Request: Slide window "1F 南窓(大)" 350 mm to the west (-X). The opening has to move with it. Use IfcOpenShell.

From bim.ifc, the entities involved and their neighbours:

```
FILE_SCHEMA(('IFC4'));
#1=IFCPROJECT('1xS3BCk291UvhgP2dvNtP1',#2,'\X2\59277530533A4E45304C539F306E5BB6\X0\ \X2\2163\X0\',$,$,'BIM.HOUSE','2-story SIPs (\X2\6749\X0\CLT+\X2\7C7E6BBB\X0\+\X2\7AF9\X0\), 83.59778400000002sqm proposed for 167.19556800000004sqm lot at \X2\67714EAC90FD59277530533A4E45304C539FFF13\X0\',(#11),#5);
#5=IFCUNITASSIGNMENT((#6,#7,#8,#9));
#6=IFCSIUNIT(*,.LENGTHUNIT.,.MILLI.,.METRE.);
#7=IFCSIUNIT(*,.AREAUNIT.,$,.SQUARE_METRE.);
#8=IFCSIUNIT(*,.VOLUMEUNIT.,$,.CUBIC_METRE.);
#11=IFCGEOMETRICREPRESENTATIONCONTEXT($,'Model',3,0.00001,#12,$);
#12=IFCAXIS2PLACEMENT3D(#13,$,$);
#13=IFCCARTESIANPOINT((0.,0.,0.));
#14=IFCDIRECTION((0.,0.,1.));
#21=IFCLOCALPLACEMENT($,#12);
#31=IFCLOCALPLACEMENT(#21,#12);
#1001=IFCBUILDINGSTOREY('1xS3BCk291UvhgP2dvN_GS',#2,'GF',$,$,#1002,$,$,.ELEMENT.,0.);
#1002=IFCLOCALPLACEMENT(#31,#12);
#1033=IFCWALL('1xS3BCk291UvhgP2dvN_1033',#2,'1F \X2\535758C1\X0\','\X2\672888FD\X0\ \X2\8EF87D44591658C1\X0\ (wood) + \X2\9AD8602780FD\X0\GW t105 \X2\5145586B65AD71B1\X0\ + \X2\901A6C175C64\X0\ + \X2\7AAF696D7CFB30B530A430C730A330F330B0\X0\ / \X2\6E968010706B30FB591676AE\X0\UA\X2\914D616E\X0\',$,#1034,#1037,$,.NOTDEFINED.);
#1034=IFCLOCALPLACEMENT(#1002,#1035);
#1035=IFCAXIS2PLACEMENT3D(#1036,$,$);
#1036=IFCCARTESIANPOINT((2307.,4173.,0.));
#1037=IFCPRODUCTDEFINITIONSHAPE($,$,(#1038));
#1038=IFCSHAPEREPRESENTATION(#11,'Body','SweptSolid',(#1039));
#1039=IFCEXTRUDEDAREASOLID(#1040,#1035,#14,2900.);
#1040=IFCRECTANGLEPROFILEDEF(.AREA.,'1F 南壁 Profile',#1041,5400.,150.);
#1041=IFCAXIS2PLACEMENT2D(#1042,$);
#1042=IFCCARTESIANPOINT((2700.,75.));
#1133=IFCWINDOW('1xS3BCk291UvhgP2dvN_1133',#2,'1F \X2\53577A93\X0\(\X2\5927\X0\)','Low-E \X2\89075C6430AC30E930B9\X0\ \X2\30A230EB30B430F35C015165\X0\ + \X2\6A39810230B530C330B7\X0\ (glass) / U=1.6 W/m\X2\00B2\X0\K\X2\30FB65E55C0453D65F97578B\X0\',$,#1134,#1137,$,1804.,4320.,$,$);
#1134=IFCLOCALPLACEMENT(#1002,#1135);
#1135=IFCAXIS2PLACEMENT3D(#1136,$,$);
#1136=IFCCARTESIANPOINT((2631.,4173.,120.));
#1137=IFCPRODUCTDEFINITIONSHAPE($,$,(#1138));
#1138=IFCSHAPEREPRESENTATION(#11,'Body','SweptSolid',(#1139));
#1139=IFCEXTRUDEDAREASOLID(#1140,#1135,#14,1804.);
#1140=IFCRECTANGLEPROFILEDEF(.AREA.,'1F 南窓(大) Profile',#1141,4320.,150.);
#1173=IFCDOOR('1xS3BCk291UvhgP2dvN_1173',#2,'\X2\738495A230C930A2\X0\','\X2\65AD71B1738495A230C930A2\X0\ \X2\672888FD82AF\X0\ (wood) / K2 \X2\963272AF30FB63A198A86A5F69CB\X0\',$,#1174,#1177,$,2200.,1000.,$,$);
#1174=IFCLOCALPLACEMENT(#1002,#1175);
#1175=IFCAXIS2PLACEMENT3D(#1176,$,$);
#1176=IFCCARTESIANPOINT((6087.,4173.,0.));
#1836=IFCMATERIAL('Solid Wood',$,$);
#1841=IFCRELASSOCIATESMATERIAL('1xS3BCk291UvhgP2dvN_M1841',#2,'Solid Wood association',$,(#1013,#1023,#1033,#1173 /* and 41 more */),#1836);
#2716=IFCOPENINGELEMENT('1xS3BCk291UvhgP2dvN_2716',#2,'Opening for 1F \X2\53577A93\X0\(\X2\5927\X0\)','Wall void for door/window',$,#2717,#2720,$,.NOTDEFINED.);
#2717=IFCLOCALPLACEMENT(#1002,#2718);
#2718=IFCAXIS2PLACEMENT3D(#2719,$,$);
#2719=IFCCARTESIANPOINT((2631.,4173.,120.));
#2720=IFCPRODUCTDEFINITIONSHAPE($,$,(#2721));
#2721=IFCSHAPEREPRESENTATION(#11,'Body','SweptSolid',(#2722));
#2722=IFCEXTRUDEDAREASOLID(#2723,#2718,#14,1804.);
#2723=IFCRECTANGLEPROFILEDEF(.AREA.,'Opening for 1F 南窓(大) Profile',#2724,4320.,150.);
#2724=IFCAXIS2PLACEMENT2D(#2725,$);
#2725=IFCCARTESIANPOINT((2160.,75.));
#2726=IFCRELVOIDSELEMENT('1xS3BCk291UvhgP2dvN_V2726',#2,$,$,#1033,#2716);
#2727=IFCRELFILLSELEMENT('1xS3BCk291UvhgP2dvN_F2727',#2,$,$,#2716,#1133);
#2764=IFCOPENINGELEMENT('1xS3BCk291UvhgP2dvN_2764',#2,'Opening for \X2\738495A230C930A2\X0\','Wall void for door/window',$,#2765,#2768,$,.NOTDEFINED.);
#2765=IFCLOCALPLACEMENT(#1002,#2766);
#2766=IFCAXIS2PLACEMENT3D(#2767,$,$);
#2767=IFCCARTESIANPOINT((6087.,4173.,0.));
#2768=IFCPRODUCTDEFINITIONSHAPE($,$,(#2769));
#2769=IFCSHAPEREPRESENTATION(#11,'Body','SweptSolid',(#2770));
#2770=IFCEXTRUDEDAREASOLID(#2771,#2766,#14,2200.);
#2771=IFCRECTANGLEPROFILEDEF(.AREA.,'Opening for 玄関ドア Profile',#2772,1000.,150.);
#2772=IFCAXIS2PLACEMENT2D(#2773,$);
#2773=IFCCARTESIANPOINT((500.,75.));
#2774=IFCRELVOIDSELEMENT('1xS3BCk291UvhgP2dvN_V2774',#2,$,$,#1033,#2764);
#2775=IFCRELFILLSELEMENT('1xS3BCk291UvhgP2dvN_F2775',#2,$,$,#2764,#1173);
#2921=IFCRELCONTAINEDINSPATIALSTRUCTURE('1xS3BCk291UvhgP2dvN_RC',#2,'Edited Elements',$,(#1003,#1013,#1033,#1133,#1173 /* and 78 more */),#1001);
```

```python
import ifcopenshell
import ifcopenshell.api.geometry
import ifcopenshell.util.placement
import ifcopenshell.util.unit

model = ifcopenshell.open("bim.ifc")
unit_scale = ifcopenshell.util.unit.calculate_unit_scale(model)

window = model.by_guid("1xS3BCk291UvhgP2dvN_1133")
opening = window.FillsVoids[0].RelatingOpeningElement
wall = opening.VoidsElements[0].RelatingBuildingElement

wall_matrix = ifcopenshell.util.placement.get_local_placement(wall.ObjectPlacement)
shift = wall_matrix[:3, 0] * -0.35 / unit_scale
before = ifcopenshell.util.placement.get_local_placement(window.ObjectPlacement)[:3, 3].copy()

# The window is not placed relative to its opening, so move both.
for product in (opening, window):
    matrix = ifcopenshell.util.placement.get_local_placement(product.ObjectPlacement)
    matrix[:3, 3] += shift
    ifcopenshell.api.geometry.edit_object_placement(model, product=product, matrix=matrix, is_si=False)

after = ifcopenshell.util.placement.get_local_placement(window.ObjectPlacement)[:3, 3]
print("window moved by", (after - before).round(3) + 0.0)

model.write("bim_v2.ifc")
```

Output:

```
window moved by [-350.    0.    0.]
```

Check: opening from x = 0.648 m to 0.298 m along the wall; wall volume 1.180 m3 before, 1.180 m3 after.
